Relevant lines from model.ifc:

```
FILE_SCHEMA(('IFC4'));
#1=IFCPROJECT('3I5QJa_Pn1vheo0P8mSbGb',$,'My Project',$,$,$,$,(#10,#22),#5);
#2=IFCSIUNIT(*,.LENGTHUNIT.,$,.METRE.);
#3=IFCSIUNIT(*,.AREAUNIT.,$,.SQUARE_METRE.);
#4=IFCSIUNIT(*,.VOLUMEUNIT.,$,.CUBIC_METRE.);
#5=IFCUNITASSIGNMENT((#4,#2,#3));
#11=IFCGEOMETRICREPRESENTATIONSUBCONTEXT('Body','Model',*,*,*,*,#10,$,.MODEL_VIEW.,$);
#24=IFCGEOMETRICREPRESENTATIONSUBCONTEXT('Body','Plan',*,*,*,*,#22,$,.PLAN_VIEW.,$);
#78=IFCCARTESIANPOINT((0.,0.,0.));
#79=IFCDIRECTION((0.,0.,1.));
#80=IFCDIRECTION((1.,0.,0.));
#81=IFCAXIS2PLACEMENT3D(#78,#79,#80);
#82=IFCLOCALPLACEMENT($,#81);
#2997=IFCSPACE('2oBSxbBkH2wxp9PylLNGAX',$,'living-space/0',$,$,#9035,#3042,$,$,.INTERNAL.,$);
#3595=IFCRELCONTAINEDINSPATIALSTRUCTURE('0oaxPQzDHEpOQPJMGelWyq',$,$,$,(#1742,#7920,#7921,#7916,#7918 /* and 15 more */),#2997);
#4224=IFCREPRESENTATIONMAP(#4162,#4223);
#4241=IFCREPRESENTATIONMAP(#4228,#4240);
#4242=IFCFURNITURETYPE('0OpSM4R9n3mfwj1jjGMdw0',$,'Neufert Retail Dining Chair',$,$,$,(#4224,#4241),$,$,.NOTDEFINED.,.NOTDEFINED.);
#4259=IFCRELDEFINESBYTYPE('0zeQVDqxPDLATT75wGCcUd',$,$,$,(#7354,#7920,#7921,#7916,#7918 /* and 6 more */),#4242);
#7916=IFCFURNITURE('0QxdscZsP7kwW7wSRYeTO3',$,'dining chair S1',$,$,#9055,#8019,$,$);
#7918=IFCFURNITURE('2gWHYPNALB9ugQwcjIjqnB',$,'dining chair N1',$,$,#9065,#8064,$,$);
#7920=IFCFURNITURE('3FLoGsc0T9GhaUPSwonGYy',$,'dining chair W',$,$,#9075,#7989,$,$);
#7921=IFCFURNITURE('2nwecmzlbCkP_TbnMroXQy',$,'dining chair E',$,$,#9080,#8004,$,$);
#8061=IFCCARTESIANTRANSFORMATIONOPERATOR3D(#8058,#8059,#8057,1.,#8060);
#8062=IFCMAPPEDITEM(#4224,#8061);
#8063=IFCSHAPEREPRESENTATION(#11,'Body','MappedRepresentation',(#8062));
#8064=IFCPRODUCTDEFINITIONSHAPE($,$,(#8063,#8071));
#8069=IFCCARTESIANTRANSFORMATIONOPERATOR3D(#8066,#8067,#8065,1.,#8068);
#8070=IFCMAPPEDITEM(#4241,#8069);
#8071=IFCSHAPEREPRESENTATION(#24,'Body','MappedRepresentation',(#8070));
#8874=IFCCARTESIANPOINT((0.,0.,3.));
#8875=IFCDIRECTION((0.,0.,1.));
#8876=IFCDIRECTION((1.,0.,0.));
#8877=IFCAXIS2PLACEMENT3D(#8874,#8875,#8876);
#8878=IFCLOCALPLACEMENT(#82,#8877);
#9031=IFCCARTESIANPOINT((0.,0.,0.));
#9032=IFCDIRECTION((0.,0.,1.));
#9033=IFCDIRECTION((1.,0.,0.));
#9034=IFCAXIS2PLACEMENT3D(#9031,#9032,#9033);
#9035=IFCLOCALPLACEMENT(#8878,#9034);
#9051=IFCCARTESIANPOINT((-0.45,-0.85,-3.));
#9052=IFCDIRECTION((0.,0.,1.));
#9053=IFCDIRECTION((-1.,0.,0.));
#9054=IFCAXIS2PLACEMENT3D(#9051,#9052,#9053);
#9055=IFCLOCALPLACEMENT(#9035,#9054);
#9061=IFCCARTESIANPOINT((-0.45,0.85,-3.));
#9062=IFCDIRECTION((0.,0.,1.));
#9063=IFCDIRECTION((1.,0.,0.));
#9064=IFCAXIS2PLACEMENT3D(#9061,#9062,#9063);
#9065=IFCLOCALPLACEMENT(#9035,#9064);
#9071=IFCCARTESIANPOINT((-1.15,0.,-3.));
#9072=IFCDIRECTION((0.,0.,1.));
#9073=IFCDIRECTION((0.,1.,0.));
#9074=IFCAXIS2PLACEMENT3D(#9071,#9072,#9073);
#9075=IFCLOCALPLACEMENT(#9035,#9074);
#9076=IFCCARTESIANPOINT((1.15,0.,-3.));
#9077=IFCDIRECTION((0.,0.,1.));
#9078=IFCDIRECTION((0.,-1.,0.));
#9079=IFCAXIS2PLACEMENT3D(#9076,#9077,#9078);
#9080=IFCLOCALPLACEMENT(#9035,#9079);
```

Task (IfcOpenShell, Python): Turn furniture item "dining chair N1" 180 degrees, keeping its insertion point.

```python
import ifcopenshell
import ifcopenshell.api.geometry
import ifcopenshell.util.placement

model = ifcopenshell.open("model.ifc")

item = model.by_guid("2gWHYPNALB9ugQwcjIjqnB")
matrix = ifcopenshell.util.placement.get_local_placement(item.ObjectPlacement)
matrix = matrix @ ifcopenshell.util.placement.rotation(180, "Z")
ifcopenshell.api.geometry.edit_object_placement(model, product=item, matrix=matrix, is_si=False)

print(ifcopenshell.util.placement.get_local_placement(item.ObjectPlacement).round(3) + 0.0)

model.write("model_rev.ifc")
```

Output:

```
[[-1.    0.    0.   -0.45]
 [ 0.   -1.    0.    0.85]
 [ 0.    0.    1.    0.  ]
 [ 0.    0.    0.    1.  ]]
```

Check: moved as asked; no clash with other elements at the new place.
